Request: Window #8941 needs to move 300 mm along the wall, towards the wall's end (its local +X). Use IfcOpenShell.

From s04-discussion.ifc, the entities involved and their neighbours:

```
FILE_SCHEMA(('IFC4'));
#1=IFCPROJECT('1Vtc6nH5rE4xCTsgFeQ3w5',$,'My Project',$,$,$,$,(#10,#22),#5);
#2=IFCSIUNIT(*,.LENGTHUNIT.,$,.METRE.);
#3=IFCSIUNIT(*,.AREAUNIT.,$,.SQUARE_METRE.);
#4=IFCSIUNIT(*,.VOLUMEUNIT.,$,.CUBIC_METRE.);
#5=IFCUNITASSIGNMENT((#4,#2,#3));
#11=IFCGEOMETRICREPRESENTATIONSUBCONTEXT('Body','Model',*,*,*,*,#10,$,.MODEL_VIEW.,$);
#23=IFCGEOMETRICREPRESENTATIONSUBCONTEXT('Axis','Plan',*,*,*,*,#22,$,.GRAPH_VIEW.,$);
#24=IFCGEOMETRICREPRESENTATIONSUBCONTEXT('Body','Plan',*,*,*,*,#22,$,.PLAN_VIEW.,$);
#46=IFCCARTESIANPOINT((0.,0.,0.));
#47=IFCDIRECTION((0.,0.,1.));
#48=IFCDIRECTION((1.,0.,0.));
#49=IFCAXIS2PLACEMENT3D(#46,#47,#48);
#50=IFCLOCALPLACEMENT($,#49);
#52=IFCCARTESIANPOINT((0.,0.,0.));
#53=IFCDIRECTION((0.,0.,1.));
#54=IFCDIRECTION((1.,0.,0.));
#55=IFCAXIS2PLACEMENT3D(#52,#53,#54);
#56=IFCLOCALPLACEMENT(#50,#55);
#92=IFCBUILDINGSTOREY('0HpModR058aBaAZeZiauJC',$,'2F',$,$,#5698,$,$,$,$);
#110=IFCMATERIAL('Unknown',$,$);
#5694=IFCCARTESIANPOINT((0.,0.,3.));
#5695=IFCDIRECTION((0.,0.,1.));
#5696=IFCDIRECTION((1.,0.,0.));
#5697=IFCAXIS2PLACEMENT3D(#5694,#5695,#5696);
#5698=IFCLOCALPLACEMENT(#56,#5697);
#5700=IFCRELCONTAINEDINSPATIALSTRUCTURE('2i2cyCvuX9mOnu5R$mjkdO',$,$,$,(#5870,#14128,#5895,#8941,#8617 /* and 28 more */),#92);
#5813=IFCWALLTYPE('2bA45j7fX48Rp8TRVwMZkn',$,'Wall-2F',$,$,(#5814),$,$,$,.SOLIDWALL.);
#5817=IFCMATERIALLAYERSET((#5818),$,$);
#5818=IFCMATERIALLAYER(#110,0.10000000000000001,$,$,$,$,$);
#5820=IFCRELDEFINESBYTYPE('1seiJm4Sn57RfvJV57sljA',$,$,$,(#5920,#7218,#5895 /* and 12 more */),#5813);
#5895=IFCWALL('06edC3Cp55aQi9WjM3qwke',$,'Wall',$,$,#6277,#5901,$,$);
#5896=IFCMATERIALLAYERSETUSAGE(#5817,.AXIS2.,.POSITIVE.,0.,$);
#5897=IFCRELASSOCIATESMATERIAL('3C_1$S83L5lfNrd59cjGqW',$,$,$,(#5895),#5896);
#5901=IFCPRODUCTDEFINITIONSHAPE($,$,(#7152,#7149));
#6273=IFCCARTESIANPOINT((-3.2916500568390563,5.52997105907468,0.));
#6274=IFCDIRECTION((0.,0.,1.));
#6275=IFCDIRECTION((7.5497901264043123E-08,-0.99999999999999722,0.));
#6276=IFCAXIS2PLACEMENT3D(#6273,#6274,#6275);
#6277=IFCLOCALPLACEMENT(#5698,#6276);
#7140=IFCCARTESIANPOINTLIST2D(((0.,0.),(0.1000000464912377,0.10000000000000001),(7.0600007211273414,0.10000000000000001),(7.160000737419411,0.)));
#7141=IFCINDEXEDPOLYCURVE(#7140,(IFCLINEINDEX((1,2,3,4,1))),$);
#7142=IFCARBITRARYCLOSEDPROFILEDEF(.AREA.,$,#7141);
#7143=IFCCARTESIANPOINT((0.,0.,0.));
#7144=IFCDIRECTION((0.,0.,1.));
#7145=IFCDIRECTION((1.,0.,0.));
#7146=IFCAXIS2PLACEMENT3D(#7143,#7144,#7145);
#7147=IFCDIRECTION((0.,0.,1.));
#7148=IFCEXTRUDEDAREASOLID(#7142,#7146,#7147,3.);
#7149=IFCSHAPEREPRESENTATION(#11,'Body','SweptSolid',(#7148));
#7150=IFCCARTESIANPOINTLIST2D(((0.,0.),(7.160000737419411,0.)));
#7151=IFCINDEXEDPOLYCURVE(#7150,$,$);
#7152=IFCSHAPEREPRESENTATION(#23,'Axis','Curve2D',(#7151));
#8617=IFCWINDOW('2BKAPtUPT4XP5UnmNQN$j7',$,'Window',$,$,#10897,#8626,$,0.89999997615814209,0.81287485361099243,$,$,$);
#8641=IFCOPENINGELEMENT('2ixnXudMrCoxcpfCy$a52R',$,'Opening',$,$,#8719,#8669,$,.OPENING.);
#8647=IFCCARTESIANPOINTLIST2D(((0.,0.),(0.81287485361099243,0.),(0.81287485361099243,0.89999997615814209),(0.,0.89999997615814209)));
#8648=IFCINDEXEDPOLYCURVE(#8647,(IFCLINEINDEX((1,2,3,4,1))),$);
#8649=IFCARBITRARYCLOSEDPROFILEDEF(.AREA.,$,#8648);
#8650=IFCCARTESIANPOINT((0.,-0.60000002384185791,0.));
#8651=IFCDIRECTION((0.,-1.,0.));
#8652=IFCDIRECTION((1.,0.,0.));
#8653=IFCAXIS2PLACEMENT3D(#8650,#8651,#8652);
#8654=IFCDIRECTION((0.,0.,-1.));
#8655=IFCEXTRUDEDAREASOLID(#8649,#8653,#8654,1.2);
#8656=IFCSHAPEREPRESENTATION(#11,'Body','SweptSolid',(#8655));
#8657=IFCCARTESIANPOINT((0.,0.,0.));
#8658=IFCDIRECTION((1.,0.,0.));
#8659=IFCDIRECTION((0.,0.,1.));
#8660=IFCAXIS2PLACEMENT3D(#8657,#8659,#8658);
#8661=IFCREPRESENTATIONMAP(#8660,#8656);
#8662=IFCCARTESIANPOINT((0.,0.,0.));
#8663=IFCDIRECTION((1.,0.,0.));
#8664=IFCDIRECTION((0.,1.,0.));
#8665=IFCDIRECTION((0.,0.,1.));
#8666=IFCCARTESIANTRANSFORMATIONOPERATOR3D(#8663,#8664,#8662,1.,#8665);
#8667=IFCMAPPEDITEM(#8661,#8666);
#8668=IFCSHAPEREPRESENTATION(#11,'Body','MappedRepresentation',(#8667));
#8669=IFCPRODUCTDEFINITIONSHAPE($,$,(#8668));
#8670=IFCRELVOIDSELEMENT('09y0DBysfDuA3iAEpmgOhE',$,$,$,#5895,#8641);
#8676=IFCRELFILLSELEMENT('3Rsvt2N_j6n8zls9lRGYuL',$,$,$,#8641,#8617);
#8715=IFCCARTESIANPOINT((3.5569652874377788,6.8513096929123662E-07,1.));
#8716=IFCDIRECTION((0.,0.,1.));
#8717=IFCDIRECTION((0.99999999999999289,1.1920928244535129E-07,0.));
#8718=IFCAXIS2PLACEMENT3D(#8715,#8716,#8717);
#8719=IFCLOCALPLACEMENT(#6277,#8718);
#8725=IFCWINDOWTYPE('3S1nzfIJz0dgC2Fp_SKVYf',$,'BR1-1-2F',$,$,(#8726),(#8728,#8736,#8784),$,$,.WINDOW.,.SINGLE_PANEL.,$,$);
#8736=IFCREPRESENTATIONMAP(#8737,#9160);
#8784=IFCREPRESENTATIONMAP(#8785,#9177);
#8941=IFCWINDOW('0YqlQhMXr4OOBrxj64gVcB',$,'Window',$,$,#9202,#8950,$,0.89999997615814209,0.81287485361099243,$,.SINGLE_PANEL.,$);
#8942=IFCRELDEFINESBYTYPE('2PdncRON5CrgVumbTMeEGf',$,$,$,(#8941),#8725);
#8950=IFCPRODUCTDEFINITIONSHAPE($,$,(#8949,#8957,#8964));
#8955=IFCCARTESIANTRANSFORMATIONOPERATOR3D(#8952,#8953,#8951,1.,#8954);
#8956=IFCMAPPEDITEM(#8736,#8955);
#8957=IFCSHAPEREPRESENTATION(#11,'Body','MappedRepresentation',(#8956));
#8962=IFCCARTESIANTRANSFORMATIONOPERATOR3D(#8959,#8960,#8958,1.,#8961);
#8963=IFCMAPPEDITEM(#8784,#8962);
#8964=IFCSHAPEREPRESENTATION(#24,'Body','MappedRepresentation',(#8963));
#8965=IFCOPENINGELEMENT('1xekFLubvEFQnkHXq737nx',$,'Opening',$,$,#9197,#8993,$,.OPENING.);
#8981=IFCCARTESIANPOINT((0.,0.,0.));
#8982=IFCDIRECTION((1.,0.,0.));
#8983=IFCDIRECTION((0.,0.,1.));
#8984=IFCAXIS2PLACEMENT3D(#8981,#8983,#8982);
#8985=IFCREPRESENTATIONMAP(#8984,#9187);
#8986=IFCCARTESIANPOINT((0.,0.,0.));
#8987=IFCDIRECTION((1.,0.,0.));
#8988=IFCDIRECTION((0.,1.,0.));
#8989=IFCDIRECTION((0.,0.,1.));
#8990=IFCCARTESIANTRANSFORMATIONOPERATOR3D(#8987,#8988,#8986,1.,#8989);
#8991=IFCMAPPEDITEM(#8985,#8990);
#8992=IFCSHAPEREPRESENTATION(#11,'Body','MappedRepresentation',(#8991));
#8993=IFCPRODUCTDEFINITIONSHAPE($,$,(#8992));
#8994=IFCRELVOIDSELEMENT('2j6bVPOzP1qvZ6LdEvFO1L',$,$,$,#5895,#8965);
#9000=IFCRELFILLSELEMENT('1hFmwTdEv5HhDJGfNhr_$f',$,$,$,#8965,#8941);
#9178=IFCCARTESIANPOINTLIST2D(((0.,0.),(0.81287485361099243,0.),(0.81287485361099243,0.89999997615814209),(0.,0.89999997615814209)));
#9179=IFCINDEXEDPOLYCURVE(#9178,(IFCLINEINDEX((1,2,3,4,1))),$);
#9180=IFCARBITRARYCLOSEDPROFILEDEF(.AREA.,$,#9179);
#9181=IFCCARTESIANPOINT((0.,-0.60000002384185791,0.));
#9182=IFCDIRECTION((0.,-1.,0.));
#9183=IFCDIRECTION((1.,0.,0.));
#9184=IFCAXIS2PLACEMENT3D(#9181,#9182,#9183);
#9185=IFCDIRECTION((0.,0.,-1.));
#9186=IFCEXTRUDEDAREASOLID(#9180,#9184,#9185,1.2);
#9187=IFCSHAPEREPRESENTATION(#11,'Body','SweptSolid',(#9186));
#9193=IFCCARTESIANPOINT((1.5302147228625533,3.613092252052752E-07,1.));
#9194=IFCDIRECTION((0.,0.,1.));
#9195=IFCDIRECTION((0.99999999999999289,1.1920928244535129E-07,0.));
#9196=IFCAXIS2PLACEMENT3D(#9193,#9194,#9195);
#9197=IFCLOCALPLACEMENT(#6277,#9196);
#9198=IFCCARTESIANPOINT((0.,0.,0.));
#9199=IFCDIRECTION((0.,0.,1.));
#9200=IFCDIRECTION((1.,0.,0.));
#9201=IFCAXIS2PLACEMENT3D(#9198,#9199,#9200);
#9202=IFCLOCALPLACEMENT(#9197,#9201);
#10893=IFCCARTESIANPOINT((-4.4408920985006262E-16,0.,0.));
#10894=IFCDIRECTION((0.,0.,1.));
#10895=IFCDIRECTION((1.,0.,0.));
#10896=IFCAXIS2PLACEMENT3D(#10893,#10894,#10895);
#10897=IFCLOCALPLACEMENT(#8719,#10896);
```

```python
import ifcopenshell
import ifcopenshell.api.geometry
import ifcopenshell.util.placement

model = ifcopenshell.open("s04-discussion.ifc")

window = model.by_guid("0YqlQhMXr4OOBrxj64gVcB")
opening = window.FillsVoids[0].RelatingOpeningElement
wall = opening.VoidsElements[0].RelatingBuildingElement

wall_matrix = ifcopenshell.util.placement.get_local_placement(wall.ObjectPlacement)
shift = wall_matrix[:3, 0] * 0.3
before = ifcopenshell.util.placement.get_local_placement(window.ObjectPlacement)[:3, 3].copy()

# The window is placed relative to its opening, so it follows when the opening moves.
matrix = ifcopenshell.util.placement.get_local_placement(opening.ObjectPlacement)
matrix[:3, 3] += shift
ifcopenshell.api.geometry.edit_object_placement(
    model, product=opening, matrix=matrix, is_si=False, should_transform_children=True
)

after = ifcopenshell.util.placement.get_local_placement(window.ObjectPlacement)[:3, 3]
print("window moved by", (after - before).round(3) + 0.0)

model.write("s04-discussion_updated.ifc")
```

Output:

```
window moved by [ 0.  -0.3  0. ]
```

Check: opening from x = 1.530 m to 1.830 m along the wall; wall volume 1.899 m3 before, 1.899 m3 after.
